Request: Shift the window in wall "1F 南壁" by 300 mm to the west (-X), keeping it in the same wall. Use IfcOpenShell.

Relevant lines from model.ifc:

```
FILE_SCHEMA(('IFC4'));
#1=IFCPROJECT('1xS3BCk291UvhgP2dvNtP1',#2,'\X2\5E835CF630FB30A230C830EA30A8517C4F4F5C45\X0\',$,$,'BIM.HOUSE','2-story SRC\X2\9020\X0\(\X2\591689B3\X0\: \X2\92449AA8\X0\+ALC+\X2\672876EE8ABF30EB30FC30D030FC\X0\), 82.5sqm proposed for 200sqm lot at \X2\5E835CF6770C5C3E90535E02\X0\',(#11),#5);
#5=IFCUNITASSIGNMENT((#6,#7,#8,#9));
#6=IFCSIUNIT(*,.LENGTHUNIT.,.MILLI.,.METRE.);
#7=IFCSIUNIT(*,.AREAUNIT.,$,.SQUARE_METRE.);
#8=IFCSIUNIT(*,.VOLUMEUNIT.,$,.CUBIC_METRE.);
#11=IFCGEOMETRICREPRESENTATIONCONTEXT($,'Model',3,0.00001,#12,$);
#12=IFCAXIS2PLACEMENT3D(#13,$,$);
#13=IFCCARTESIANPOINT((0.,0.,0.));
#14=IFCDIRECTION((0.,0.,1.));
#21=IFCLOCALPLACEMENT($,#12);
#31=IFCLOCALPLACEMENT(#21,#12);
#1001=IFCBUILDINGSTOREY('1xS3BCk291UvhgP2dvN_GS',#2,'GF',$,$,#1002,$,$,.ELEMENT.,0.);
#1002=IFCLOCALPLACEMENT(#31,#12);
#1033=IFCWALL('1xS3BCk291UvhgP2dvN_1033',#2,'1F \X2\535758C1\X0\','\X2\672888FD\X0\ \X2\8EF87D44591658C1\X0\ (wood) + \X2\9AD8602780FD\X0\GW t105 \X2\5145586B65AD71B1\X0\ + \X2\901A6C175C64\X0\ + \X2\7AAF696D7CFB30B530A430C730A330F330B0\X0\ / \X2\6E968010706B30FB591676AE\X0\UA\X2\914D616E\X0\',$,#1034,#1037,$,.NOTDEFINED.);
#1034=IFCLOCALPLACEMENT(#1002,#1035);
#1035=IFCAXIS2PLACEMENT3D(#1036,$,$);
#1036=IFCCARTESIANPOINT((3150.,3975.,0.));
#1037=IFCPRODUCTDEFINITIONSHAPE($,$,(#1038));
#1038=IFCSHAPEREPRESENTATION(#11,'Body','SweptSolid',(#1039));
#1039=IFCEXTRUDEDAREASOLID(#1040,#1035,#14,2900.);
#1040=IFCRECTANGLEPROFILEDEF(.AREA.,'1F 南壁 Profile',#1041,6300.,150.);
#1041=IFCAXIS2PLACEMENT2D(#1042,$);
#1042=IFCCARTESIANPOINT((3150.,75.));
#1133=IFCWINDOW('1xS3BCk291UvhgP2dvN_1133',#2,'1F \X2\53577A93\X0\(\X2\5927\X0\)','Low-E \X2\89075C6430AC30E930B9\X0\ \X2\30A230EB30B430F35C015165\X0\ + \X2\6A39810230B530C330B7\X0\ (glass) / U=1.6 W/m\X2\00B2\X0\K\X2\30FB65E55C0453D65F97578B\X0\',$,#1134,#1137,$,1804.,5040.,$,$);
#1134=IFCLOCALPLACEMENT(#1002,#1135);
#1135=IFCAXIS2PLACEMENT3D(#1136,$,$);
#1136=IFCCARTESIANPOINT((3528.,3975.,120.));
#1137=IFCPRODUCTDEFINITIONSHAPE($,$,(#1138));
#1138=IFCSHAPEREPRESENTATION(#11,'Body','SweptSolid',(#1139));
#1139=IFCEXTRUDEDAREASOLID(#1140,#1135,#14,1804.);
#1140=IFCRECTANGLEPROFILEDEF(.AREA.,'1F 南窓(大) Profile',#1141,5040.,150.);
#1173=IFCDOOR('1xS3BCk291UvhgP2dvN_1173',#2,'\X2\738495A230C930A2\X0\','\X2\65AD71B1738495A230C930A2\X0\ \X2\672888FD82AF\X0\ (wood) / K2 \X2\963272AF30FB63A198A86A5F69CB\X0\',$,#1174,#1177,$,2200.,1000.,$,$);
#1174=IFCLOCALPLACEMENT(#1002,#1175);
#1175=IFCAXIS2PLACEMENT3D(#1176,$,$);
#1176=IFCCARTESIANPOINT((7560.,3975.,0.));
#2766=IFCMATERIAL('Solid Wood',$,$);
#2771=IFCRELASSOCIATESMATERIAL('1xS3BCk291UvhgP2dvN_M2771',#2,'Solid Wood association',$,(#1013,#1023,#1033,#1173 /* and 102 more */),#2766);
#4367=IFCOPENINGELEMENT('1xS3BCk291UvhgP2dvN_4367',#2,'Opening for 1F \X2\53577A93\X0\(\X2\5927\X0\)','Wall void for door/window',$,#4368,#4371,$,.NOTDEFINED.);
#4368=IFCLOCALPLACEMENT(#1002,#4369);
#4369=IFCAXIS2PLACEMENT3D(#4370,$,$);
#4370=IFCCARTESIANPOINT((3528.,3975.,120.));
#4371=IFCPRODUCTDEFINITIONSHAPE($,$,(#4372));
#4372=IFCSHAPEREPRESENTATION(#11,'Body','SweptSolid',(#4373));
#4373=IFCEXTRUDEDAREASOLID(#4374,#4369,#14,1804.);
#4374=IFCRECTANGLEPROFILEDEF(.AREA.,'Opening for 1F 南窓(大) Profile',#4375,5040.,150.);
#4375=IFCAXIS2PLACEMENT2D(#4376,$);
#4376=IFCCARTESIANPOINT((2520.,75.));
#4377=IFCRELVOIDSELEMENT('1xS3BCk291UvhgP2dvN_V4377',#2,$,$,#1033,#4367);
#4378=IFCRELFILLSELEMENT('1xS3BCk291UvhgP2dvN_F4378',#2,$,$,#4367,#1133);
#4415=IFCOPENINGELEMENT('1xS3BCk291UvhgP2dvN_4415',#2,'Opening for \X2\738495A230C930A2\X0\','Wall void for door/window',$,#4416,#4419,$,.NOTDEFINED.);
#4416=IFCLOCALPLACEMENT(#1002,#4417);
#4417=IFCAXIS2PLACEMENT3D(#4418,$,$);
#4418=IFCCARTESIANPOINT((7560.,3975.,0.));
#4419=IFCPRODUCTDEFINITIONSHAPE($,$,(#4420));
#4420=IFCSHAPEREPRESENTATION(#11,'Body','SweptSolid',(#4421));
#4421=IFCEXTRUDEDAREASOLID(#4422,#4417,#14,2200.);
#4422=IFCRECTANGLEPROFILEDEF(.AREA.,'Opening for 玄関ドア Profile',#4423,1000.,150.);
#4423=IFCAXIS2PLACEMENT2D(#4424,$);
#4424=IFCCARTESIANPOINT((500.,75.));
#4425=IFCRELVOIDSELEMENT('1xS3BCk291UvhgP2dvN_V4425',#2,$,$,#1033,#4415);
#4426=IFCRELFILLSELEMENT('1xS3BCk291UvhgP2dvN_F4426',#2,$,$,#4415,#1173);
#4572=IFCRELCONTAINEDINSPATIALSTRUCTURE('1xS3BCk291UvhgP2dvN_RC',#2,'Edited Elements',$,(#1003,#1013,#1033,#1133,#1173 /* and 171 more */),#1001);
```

```python
import ifcopenshell
import ifcopenshell.api.geometry
import ifcopenshell.util.placement
import ifcopenshell.util.unit

model = ifcopenshell.open("model.ifc")
unit_scale = ifcopenshell.util.unit.calculate_unit_scale(model)

window = model.by_guid("1xS3BCk291UvhgP2dvN_1133")
opening = window.FillsVoids[0].RelatingOpeningElement
wall = opening.VoidsElements[0].RelatingBuildingElement

wall_matrix = ifcopenshell.util.placement.get_local_placement(wall.ObjectPlacement)
shift = wall_matrix[:3, 0] * -0.3 / unit_scale
before = ifcopenshell.util.placement.get_local_placement(window.ObjectPlacement)[:3, 3].copy()

# The window is not placed relative to its opening, so move both.
for product in (opening, window):
    matrix = ifcopenshell.util.placement.get_local_placement(product.ObjectPlacement)
    matrix[:3, 3] += shift
    ifcopenshell.api.geometry.edit_object_placement(model, product=product, matrix=matrix, is_si=False)

after = ifcopenshell.util.placement.get_local_placement(window.ObjectPlacement)[:3, 3]
print("window moved by", (after - before).round(3) + 0.0)

model.write("model_edited.ifc")
```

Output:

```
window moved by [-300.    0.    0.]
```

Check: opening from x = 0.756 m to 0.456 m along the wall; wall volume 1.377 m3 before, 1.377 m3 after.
